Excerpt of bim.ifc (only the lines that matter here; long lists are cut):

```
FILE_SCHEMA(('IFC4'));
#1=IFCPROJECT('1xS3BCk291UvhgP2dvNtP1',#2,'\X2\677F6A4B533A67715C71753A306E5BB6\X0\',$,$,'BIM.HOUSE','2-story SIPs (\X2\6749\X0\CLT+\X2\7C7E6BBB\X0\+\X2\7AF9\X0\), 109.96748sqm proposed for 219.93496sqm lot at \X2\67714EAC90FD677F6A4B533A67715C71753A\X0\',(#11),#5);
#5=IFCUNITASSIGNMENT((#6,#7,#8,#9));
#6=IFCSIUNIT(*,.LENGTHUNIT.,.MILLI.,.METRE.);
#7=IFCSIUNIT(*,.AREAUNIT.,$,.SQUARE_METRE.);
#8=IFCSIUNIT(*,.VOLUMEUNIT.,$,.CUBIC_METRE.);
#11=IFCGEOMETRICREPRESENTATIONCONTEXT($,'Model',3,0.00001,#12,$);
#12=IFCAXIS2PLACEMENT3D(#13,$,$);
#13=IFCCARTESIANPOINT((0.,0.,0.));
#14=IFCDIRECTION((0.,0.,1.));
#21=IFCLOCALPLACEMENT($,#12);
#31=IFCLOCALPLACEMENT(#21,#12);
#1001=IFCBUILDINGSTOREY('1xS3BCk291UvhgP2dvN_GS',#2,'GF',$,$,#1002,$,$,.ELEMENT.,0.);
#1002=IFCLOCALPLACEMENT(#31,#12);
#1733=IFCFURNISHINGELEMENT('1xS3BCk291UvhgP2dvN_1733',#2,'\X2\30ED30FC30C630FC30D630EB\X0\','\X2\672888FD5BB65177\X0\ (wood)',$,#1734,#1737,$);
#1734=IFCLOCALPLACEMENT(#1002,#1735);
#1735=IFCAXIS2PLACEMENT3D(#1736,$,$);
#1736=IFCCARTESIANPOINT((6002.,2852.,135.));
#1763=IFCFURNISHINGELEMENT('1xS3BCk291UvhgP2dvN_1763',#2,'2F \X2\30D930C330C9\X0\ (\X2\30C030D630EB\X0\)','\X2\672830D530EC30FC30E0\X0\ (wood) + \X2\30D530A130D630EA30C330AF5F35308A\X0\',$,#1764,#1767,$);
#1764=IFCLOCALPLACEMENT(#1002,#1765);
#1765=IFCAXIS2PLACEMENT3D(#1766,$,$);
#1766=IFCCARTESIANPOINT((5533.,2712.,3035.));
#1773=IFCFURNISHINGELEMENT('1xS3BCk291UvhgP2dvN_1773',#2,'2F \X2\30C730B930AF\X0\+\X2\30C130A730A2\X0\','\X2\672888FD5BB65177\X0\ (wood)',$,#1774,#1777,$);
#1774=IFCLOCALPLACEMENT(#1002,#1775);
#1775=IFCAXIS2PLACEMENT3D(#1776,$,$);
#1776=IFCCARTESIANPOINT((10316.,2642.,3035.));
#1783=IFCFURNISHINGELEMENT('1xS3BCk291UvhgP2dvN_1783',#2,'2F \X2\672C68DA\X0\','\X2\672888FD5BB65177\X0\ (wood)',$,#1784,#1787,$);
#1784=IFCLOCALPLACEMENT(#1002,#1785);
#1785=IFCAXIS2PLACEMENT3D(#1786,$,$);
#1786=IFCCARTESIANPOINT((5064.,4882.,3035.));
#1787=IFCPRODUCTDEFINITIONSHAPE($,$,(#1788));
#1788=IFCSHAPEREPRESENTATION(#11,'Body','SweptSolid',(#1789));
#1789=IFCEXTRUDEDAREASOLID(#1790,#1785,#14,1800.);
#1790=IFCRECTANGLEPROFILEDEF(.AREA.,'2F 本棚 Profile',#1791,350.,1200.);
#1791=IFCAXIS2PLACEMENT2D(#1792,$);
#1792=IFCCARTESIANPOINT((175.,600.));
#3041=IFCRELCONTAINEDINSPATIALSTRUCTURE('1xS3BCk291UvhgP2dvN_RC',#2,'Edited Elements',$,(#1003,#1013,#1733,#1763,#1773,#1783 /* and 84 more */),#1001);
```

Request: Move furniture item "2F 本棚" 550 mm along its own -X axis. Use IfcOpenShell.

```python
import ifcopenshell
import ifcopenshell.api.geometry
import ifcopenshell.util.placement
import ifcopenshell.util.unit

model = ifcopenshell.open("bim.ifc")
unit_scale = ifcopenshell.util.unit.calculate_unit_scale(model)

item = model.by_guid("1xS3BCk291UvhgP2dvN_1783")
matrix = ifcopenshell.util.placement.get_local_placement(item.ObjectPlacement)
matrix[:3, 3] -= matrix[:3, 0] * 0.55 / unit_scale
ifcopenshell.api.geometry.edit_object_placement(model, product=item, matrix=matrix, is_si=False)

print(ifcopenshell.util.placement.get_local_placement(item.ObjectPlacement).round(3) + 0.0)

model.write("bim_edited.ifc")
```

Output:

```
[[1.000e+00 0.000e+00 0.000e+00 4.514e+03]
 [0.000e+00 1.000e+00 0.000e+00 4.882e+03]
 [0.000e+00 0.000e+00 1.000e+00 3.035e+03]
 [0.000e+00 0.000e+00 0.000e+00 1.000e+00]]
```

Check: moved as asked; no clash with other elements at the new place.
